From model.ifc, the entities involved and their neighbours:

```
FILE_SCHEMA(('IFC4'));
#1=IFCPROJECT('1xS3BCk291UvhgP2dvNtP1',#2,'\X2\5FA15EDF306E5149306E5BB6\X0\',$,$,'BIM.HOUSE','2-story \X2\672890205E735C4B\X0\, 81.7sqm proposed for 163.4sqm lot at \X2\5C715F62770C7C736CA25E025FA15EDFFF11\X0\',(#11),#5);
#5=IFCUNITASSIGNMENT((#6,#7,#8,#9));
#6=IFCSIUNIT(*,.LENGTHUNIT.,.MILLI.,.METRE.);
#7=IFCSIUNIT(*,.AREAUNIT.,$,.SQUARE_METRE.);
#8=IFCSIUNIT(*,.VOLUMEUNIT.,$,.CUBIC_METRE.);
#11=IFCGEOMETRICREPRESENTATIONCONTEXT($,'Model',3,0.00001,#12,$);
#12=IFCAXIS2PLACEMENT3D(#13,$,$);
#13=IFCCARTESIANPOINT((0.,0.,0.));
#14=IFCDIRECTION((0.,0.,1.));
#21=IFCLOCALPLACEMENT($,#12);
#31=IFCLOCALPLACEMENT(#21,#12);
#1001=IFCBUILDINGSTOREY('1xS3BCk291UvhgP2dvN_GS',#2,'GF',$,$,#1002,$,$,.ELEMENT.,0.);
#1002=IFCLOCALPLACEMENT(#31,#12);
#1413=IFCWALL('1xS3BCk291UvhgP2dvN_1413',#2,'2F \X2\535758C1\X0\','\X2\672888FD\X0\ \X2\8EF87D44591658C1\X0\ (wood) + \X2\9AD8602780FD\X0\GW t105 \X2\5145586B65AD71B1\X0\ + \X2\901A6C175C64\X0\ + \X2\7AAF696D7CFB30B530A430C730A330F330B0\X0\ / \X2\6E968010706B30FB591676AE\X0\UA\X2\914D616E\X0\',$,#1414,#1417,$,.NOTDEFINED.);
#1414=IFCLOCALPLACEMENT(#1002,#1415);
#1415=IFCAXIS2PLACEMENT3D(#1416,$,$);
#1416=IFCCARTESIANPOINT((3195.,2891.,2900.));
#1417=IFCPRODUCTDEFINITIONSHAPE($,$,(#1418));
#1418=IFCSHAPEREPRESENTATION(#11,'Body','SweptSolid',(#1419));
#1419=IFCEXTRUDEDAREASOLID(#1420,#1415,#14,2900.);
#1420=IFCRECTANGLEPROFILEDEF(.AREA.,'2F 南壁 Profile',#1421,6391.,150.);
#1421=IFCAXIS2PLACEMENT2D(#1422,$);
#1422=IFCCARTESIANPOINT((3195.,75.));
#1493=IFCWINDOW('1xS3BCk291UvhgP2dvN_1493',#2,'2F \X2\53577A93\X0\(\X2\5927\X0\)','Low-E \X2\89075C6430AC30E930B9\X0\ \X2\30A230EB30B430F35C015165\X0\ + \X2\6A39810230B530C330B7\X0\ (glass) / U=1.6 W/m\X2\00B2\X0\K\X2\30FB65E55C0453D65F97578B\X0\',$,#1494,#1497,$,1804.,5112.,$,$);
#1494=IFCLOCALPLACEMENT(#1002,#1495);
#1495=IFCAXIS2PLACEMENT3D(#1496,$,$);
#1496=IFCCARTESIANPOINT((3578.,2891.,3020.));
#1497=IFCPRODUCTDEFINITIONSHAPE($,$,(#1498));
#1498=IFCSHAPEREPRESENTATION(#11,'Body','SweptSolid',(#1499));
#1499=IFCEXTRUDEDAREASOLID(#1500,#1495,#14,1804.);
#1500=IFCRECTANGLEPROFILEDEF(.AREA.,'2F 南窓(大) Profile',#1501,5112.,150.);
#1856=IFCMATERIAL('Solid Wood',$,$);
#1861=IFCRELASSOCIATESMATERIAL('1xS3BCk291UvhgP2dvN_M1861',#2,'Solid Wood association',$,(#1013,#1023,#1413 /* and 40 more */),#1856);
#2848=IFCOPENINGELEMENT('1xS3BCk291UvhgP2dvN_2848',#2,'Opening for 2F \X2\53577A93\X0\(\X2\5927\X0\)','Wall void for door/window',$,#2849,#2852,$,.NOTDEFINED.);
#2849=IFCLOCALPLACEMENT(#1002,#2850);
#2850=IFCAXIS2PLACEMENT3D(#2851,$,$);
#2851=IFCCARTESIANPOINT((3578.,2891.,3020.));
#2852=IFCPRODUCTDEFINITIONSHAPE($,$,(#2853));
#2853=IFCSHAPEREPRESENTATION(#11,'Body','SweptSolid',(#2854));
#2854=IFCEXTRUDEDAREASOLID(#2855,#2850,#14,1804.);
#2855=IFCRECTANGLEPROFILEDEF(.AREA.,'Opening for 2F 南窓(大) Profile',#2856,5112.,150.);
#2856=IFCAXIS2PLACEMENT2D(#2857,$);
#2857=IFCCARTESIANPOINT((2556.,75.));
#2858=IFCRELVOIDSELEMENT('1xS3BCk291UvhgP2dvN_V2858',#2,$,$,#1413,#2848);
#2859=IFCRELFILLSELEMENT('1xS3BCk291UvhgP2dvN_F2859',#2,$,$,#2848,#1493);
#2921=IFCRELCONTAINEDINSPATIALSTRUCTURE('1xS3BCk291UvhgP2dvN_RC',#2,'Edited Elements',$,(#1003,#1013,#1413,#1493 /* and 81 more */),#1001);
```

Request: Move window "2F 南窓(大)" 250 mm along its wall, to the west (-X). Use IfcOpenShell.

```python
import ifcopenshell
import ifcopenshell.api.geometry
import ifcopenshell.util.placement

model = ifcopenshell.open("model.ifc")

window = model.by_id(1493)
opening = window.FillsVoids[0].RelatingOpeningElement
wall = opening.VoidsElements[0].RelatingBuildingElement

wall_matrix = ifcopenshell.util.placement.get_local_placement(wall.ObjectPlacement)
shift = wall_matrix[:3, 0] * -250.0
before = ifcopenshell.util.placement.get_local_placement(window.ObjectPlacement)[:3, 3].copy()

# The window is not placed relative to its opening, so move both.
for product in (opening, window):
    matrix = ifcopenshell.util.placement.get_local_placement(product.ObjectPlacement)
    matrix[:3, 3] += shift
    ifcopenshell.api.geometry.edit_object_placement(model, product=product, matrix=matrix, is_si=False)

after = ifcopenshell.util.placement.get_local_placement(window.ObjectPlacement)[:3, 3]
print("window moved by", (after - before).round(3) + 0.0)

model.write("model_edited.ifc")
```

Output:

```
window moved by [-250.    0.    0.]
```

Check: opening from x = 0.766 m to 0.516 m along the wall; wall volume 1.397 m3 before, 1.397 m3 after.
